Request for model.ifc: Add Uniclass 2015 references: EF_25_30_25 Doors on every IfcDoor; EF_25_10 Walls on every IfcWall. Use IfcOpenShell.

First a look at what the model holds.

```python
import ifcopenshell

model = ifcopenshell.open("model.ifc")
print(model.schema)
print("classifications:", [c.Name for c in model.by_type("IfcClassification")])
for ifc_class in ("IfcDoor", "IfcRoof", "IfcStair", "IfcWall", "IfcWindow"):
    print(ifc_class, len(model.by_type(ifc_class)))
```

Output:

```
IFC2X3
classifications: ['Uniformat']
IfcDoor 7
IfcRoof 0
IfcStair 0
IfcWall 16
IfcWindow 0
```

```python
import ifcopenshell
import ifcopenshell.api.classification

model = ifcopenshell.open("model.ifc")

# IFC2X3 requires Source and Edition and has no link from the project to the system.
system = model.create_entity("IfcClassification", Source="NBS", Edition="2015", Name="Uniclass 2015")

codes = {
    "IfcDoor": ("EF_25_30_25", "Doors"),
    "IfcWall": ("EF_25_10", "Walls"),
}
for ifc_class, (code, name) in codes.items():
    products = model.by_type(ifc_class)
    ifcopenshell.api.classification.add_reference(
        model, products=products, classification=system, identification=code, name=name
    )
    print(code, len(products))

model.write("model-out.ifc")
```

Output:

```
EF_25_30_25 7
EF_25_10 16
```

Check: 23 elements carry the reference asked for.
